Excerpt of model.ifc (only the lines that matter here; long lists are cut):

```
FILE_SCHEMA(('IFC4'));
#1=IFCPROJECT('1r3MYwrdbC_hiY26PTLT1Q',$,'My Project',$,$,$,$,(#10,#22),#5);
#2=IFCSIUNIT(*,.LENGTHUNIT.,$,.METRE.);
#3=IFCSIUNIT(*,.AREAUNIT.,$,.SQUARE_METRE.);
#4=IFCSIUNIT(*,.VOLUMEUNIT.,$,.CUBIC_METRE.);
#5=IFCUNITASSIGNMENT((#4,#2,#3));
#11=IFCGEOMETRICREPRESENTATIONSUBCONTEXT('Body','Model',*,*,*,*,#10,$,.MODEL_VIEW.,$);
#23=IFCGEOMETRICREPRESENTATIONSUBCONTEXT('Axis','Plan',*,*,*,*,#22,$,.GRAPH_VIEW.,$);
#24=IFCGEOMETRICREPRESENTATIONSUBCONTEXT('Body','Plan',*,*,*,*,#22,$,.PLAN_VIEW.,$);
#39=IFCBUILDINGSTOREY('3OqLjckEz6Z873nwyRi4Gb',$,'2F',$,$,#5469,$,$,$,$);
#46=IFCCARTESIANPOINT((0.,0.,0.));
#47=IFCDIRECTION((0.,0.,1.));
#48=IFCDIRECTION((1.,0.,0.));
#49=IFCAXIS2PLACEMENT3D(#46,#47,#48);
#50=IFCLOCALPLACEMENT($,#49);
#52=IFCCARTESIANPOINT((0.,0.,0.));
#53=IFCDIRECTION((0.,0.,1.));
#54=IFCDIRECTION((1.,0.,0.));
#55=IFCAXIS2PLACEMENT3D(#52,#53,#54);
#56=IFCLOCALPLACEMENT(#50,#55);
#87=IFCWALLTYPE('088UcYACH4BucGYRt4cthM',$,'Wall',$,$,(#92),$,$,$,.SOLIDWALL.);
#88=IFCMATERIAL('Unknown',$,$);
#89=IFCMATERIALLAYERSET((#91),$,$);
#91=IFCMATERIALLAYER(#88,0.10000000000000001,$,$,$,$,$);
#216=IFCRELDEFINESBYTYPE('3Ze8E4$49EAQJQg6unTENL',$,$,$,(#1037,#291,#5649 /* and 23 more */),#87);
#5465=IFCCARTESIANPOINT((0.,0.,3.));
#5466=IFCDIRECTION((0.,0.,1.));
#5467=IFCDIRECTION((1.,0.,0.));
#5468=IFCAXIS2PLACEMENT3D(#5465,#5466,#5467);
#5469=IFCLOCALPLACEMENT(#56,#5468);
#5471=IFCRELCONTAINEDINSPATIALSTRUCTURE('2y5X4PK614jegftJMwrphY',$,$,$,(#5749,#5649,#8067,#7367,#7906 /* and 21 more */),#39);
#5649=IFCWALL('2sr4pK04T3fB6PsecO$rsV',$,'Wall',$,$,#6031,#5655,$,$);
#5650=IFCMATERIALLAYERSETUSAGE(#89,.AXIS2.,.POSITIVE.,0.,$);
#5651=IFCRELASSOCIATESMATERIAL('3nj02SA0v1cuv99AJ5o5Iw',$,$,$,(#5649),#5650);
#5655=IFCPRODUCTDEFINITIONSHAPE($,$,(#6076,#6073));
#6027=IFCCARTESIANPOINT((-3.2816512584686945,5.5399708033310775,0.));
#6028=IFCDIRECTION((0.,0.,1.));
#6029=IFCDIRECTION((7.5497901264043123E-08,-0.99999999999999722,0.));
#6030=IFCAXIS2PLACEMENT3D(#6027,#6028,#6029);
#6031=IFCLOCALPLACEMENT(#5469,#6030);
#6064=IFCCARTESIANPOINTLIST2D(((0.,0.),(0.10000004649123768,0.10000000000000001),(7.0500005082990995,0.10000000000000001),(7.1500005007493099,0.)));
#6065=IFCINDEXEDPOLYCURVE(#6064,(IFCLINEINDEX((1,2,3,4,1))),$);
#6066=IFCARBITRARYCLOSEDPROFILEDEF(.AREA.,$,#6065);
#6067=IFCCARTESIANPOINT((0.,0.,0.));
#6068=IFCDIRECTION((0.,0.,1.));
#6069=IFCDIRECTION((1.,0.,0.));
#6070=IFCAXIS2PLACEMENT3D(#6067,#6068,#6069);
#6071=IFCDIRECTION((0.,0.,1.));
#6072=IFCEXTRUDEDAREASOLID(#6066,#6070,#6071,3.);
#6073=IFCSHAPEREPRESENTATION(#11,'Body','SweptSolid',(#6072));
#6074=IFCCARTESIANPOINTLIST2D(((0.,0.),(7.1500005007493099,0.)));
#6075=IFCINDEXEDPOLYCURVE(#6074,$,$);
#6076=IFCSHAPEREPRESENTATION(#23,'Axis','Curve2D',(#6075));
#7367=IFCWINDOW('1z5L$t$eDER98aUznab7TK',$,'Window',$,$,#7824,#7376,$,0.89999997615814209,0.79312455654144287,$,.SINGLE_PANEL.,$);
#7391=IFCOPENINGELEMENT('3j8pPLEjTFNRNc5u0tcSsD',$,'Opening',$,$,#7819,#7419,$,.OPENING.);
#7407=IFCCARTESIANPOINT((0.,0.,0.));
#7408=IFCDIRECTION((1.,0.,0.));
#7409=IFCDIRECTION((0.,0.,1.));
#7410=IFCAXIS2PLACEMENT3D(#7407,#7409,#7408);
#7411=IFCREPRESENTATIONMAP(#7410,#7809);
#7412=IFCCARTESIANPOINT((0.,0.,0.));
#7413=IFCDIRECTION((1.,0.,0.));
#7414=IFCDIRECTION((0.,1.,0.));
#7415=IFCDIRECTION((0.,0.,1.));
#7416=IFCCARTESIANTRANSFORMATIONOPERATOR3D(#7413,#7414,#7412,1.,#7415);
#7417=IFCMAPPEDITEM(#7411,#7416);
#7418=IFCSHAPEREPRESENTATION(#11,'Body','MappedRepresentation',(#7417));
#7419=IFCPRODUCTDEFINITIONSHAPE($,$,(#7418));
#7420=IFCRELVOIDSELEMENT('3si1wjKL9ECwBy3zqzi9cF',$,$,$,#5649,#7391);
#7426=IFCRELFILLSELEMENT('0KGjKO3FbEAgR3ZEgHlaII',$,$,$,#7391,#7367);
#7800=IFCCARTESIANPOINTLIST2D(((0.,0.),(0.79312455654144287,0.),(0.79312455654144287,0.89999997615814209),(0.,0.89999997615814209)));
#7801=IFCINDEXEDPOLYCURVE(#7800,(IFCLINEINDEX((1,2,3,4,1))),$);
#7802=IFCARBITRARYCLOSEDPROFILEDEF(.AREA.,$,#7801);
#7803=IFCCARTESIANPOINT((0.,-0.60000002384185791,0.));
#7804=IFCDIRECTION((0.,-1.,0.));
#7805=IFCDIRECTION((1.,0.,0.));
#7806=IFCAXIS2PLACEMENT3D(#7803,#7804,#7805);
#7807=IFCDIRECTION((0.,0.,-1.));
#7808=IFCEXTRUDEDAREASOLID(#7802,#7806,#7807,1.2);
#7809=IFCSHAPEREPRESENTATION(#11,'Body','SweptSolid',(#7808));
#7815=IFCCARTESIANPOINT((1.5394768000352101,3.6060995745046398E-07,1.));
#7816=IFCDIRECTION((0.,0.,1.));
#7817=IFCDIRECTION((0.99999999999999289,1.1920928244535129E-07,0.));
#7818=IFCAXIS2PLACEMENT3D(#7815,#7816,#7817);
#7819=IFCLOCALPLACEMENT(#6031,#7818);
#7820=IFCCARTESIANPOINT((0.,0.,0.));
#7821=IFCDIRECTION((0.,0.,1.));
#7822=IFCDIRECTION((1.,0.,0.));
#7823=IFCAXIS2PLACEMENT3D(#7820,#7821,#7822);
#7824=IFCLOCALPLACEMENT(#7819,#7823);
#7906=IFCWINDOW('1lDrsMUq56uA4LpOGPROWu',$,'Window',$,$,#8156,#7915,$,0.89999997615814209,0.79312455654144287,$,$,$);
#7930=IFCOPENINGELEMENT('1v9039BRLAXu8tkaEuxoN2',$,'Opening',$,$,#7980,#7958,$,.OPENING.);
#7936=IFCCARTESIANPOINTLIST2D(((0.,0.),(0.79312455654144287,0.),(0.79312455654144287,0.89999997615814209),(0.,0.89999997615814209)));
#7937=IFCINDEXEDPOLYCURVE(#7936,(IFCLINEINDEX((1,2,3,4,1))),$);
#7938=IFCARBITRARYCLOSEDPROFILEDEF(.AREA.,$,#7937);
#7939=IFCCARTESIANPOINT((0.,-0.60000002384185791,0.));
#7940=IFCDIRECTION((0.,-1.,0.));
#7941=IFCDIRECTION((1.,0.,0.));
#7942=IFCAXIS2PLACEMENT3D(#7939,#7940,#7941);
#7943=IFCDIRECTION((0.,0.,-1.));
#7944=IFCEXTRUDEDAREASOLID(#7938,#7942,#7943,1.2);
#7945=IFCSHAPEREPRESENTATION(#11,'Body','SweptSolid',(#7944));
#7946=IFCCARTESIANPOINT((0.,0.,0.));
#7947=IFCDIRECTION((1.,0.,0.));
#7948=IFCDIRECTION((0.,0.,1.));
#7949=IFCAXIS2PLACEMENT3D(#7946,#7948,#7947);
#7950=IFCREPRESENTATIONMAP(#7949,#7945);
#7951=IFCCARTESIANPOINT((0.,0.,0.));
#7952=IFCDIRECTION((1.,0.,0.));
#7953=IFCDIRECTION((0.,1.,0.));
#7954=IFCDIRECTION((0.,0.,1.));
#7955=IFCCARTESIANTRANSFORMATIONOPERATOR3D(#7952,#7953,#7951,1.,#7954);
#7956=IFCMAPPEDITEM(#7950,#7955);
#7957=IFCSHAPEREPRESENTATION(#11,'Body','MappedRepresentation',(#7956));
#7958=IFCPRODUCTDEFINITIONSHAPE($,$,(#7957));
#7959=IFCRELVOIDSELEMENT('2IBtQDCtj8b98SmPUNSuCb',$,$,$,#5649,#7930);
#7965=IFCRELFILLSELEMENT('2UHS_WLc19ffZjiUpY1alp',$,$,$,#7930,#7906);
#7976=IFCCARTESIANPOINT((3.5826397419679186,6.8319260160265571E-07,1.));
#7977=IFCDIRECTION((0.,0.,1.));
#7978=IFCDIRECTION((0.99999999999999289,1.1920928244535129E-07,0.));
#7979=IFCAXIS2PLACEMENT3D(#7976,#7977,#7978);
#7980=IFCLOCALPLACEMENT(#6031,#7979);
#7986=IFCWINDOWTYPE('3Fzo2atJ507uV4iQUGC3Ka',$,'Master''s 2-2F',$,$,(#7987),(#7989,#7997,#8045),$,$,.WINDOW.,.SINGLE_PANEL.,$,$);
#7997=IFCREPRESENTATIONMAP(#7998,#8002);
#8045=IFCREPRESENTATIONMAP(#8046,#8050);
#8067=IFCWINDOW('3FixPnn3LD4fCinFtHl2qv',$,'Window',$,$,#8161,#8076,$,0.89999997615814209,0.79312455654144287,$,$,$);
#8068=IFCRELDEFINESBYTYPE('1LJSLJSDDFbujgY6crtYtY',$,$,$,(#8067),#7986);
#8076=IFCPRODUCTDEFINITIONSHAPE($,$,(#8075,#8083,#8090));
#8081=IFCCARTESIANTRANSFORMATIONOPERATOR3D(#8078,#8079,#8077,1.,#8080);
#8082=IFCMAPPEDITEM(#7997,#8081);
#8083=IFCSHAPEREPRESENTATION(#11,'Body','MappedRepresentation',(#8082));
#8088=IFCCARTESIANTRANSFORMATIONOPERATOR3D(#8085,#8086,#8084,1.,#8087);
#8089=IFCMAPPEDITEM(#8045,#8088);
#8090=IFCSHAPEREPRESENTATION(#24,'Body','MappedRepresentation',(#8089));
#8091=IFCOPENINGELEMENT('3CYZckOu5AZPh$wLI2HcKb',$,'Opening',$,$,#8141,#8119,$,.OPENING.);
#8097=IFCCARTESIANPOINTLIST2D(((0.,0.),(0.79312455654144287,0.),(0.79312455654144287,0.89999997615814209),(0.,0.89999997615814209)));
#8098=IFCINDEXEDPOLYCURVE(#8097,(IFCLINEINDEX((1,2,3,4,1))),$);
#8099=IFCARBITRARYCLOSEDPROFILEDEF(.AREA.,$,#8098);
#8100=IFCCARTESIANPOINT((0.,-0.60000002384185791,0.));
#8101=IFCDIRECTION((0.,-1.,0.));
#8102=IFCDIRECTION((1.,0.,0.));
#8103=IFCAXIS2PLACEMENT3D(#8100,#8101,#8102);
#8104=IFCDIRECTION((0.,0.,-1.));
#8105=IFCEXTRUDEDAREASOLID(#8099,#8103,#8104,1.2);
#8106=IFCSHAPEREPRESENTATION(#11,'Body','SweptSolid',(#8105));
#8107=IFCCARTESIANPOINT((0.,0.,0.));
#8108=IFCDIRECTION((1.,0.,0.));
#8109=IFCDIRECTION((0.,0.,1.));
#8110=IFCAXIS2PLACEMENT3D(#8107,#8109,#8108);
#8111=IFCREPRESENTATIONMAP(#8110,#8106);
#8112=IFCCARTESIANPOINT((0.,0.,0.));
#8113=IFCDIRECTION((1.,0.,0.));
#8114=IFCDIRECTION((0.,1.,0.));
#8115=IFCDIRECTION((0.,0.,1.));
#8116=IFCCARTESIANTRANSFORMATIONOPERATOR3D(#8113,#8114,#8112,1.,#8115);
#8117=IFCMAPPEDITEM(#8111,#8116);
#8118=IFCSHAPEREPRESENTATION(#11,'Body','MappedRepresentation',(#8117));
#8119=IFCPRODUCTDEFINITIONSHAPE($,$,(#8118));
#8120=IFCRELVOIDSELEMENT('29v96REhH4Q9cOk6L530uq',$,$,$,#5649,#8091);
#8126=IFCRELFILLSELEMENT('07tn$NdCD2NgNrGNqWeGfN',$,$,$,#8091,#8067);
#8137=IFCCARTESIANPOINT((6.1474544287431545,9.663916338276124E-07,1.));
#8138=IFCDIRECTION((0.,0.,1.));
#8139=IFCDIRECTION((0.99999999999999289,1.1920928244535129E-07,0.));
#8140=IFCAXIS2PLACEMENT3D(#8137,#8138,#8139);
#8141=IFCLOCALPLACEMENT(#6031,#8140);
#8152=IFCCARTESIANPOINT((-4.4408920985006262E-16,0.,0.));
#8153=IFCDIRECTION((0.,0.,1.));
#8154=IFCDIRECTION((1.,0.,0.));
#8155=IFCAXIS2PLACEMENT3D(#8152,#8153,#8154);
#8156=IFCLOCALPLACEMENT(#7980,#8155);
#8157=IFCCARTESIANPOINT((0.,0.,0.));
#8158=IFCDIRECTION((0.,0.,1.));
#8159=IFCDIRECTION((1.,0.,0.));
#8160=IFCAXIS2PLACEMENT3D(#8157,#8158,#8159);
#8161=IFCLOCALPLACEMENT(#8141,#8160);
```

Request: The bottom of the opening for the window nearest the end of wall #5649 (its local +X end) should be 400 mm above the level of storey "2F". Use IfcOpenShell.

```python
import numpy as np
import ifcopenshell
import ifcopenshell.api.geometry
import ifcopenshell.geom
import ifcopenshell.util.element
import ifcopenshell.util.placement
import ifcopenshell.util.shape
import ifcopenshell.util.unit

model = ifcopenshell.open("model.ifc")
unit_scale = ifcopenshell.util.unit.calculate_unit_scale(model)

window = model.by_guid("3FixPnn3LD4fCinFtHl2qv")
opening = window.FillsVoids[0].RelatingOpeningElement
storey = ifcopenshell.util.element.get_container(window, ifc_class="IfcBuildingStorey")
level = ifcopenshell.util.placement.get_local_placement(storey.ObjectPlacement)[2, 3]

# The opening's origin need not be at the sill, so measure its lowest point.
shape = ifcopenshell.geom.create_shape(ifcopenshell.geom.settings(), opening)
bottom = ifcopenshell.util.shape.get_shape_bottom_elevation(shape, shape.geometry) / unit_scale
dz = level + 0.4 - bottom

shift = np.array([0.0, 0.0, dz])
# The window is placed relative to its opening, so it follows when the opening moves.
matrix = ifcopenshell.util.placement.get_local_placement(opening.ObjectPlacement)
matrix[:3, 3] += shift
ifcopenshell.api.geometry.edit_object_placement(
    model, product=opening, matrix=matrix, is_si=False, should_transform_children=True
)

print(f"moved by {dz * unit_scale:+.3f} m")

model.write("model-out.ifc")
```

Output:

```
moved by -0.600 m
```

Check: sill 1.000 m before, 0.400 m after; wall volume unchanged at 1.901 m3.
